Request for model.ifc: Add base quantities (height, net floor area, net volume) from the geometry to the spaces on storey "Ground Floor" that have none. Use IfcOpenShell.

First a look at what the model holds.

```python
import ifcopenshell
import ifcopenshell.util.element
import ifcopenshell.util.unit

model = ifcopenshell.open("model.ifc")
print(model.schema)
for unit_type in ("LENGTHUNIT", "AREAUNIT", "VOLUMEUNIT"):
    print(unit_type, ifcopenshell.util.unit.calculate_unit_scale(model, unit_type))
storey = next(s for s in model.by_type("IfcBuildingStorey") if s.Name == "Ground Floor")
spaces = [e for e in ifcopenshell.util.element.get_decomposition(storey) if e.is_a("IfcSpace")]
for e in sorted(spaces, key=lambda e: e.id()):
    print(e.id(), e.is_a(), e.Name, list(ifcopenshell.util.element.get_psets(e, qtos_only=True)), sep=" | ")
```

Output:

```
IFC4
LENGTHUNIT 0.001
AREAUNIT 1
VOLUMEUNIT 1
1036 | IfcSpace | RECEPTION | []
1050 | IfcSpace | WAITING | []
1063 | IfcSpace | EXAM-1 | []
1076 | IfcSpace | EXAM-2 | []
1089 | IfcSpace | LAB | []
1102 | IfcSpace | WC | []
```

```python
import ifcopenshell
import ifcopenshell.api.pset
import ifcopenshell.geom
import ifcopenshell.util.element
import ifcopenshell.util.shape
import ifcopenshell.util.unit

model = ifcopenshell.open("model.ifc")
unit_scale = ifcopenshell.util.unit.calculate_unit_scale(model)
area_scale = ifcopenshell.util.unit.calculate_unit_scale(model, "AREAUNIT")
volume_scale = ifcopenshell.util.unit.calculate_unit_scale(model, "VOLUMEUNIT")
settings = ifcopenshell.geom.settings()

storey = next(s for s in model.by_type("IfcBuildingStorey") if s.Name == "Ground Floor")
spaces = [e for e in ifcopenshell.util.element.get_decomposition(storey) if e.is_a("IfcSpace")]

for e in sorted(spaces, key=lambda e: e.id()):
    if ifcopenshell.util.element.get_psets(e, qtos_only=True, should_inherit=False):
        continue
    # Geometry comes back in metres, in the element's own axes.
    shape = ifcopenshell.geom.create_shape(settings, e)
    values = {
        "Height": ifcopenshell.util.shape.get_z(shape.geometry) / unit_scale,
        "NetFloorArea": ifcopenshell.util.shape.get_footprint_area(shape.geometry) / area_scale,
        "NetVolume": ifcopenshell.util.shape.get_volume(shape.geometry) / volume_scale,
    }
    qto = ifcopenshell.api.pset.add_qto(model, product=e, name="Qto_SpaceBaseQuantities")
    ifcopenshell.api.pset.edit_qto(model, qto=qto, properties=values)
    print(e.id(), {k: round(v, 3) for k, v in values.items()})

model.write("model_v2.ifc")
```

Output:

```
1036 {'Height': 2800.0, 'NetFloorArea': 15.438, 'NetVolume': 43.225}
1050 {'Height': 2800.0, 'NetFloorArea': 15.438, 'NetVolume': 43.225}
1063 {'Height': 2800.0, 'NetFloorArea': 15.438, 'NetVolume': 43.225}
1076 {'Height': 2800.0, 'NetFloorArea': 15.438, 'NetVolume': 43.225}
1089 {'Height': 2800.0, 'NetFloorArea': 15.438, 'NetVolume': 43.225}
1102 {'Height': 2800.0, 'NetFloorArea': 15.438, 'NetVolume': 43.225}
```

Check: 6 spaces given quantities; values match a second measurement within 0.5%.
